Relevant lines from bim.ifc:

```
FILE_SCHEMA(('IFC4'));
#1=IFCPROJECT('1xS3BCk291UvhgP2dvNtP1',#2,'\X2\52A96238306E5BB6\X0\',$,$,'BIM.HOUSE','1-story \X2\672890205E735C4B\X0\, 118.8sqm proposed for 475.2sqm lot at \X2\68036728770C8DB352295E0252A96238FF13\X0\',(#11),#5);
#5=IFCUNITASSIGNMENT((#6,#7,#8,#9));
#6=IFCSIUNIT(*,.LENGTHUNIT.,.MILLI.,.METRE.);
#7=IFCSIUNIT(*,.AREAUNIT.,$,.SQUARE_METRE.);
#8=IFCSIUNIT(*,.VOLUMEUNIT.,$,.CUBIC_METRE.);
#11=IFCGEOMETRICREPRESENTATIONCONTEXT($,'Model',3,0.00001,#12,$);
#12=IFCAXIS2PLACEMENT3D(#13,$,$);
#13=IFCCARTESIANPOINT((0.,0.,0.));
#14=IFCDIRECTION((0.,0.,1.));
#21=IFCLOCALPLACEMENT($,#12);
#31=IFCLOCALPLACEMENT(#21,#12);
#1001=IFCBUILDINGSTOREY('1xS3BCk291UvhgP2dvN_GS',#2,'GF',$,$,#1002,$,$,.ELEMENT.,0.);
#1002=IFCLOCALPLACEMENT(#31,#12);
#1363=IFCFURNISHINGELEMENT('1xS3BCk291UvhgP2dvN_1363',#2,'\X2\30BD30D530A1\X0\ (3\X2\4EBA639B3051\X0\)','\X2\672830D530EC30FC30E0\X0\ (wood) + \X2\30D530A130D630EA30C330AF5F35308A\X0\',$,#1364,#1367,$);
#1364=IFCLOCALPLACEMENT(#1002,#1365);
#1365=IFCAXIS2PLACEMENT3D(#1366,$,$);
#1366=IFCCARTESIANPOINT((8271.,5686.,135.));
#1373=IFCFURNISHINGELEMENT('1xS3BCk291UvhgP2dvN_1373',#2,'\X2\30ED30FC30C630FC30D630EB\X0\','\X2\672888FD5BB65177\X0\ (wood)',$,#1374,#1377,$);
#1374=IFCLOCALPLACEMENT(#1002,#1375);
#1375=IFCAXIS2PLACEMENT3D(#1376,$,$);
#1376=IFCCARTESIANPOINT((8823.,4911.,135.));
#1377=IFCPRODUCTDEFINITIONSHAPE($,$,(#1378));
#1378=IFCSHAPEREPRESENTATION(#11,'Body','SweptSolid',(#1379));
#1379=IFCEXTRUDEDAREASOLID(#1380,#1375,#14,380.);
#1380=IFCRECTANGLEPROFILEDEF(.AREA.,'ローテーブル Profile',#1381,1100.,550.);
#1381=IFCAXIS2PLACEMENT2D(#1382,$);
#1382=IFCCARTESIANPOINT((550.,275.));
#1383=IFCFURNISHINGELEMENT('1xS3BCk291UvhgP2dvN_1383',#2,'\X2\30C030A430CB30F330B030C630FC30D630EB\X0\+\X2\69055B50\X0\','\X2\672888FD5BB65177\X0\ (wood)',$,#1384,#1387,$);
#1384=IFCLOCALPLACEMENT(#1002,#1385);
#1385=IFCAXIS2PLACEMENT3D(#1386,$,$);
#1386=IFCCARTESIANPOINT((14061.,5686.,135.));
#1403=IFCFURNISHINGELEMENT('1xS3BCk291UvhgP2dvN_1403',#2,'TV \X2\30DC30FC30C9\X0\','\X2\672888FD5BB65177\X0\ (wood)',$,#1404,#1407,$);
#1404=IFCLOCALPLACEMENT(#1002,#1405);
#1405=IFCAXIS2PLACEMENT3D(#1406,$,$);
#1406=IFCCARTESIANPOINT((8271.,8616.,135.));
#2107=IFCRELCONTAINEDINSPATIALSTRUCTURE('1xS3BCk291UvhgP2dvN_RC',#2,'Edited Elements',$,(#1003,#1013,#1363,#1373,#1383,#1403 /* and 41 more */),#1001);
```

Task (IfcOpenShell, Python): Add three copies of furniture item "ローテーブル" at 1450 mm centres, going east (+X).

```python
import numpy as np
import ifcopenshell
import ifcopenshell.api.geometry
import ifcopenshell.api.root
import ifcopenshell.util.element
import ifcopenshell.util.placement
import ifcopenshell.util.unit

model = ifcopenshell.open("bim.ifc")
unit_scale = ifcopenshell.util.unit.calculate_unit_scale(model)


def reuse_history(source, copy):
    """copy_class also copies each property set's owner history, people and application; keep the originals."""
    for rel in copy.IsDefinedBy:
        if rel.is_a("IfcRelDefinesByProperties") and (history := rel.RelatingPropertyDefinition.OwnerHistory):
            rel.RelatingPropertyDefinition.OwnerHistory = source.OwnerHistory
            ifcopenshell.util.element.remove_deep2(model, history)


source = model.by_guid("1xS3BCk291UvhgP2dvN_1373")
base = ifcopenshell.util.placement.get_local_placement(source.ObjectPlacement)
step = np.array([1.0, 0.0, 0.0]) * 1.45 / unit_scale

for i in range(1, 4):
    copy = ifcopenshell.api.root.copy_class(model, product=source)
    copy.Representation = ifcopenshell.util.element.copy_deep(
        model, source.Representation, exclude=["IfcGeometricRepresentationContext", "IfcRepresentationMap"]
    )
    reuse_history(source, copy)
    matrix = base.copy()
    matrix[:3, 3] += i * step
    print("added at", matrix[:3, 3].round(3) + 0.0)
    ifcopenshell.api.geometry.edit_object_placement(model, product=copy, matrix=matrix, is_si=False)

model.write("bim_edited.ifc")
```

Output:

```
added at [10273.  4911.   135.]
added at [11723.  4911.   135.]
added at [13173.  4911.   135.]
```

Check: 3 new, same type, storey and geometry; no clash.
